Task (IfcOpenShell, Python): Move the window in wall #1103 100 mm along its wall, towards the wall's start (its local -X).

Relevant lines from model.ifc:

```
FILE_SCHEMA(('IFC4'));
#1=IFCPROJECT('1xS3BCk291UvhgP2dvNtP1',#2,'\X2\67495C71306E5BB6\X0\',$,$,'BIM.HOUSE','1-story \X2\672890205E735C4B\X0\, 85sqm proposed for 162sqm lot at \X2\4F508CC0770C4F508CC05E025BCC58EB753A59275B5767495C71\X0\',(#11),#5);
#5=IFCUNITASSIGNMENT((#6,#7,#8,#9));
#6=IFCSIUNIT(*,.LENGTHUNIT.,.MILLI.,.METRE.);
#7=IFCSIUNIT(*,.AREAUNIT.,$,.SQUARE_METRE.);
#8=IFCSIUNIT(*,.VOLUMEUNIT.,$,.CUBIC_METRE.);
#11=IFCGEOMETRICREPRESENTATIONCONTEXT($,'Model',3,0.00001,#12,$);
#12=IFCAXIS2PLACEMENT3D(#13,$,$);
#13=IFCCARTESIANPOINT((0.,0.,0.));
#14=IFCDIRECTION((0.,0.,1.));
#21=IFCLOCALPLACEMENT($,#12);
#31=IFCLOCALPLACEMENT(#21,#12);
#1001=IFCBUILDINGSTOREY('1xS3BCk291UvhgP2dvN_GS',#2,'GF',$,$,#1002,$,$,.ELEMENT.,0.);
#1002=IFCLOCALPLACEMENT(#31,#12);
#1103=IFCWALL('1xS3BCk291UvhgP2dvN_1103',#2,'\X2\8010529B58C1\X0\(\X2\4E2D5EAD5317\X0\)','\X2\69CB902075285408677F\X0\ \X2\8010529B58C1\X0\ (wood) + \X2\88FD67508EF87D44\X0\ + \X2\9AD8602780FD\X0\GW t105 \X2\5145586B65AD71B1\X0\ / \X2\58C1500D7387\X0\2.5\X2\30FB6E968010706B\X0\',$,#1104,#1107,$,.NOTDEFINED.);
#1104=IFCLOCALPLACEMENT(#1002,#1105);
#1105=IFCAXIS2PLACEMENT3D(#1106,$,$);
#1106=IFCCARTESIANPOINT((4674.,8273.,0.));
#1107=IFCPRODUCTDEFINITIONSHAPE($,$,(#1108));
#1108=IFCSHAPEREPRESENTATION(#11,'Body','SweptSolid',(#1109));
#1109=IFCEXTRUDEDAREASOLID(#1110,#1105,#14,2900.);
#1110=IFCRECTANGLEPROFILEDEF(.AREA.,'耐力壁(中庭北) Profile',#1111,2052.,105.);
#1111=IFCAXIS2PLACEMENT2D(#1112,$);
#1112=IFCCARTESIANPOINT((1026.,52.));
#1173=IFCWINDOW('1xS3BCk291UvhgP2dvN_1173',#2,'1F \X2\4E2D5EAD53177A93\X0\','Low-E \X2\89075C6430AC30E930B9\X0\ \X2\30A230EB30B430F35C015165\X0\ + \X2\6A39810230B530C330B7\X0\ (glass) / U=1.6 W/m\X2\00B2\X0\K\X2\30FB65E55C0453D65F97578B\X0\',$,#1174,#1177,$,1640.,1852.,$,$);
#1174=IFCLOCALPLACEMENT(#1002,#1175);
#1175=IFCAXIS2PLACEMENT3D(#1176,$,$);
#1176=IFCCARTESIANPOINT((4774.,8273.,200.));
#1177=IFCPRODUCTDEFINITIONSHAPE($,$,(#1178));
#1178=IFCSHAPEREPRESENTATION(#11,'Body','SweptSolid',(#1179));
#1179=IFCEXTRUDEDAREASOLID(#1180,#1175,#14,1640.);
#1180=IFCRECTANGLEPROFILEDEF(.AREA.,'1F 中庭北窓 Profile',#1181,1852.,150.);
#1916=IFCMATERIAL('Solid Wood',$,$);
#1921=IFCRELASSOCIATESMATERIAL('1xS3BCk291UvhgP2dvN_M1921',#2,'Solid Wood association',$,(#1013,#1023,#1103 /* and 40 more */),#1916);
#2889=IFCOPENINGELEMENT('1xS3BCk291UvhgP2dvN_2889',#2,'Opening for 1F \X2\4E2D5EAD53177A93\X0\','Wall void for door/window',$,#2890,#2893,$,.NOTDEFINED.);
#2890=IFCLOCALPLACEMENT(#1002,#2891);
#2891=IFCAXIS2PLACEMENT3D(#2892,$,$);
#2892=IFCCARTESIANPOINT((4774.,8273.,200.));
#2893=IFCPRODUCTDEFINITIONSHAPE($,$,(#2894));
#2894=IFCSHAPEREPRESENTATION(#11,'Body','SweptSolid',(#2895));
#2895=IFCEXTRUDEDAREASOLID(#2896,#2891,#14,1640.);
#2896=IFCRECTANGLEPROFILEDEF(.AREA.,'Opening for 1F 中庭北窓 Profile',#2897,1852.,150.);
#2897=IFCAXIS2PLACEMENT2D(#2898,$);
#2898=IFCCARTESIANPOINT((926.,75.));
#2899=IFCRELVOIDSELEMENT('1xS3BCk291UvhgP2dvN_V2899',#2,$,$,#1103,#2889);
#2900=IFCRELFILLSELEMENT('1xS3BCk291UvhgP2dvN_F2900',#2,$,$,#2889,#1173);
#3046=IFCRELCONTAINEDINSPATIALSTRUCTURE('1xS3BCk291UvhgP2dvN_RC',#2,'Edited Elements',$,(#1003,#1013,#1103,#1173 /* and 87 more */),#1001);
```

```python
import ifcopenshell
import ifcopenshell.api.geometry
import ifcopenshell.util.placement

model = ifcopenshell.open("model.ifc")

window = model.by_guid("1xS3BCk291UvhgP2dvN_1173")
opening = window.FillsVoids[0].RelatingOpeningElement
wall = opening.VoidsElements[0].RelatingBuildingElement

wall_matrix = ifcopenshell.util.placement.get_local_placement(wall.ObjectPlacement)
shift = wall_matrix[:3, 0] * -100.0
before = ifcopenshell.util.placement.get_local_placement(window.ObjectPlacement)[:3, 3].copy()

# The window is not placed relative to its opening, so move both.
for product in (opening, window):
    matrix = ifcopenshell.util.placement.get_local_placement(product.ObjectPlacement)
    matrix[:3, 3] += shift
    ifcopenshell.api.geometry.edit_object_placement(model, product=product, matrix=matrix, is_si=False)

after = ifcopenshell.util.placement.get_local_placement(window.ObjectPlacement)[:3, 3]
print("window moved by", (after - before).round(3) + 0.0)

model.write("model_rev.ifc")
```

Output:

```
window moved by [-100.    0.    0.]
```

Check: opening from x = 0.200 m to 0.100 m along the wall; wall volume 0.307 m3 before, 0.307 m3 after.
